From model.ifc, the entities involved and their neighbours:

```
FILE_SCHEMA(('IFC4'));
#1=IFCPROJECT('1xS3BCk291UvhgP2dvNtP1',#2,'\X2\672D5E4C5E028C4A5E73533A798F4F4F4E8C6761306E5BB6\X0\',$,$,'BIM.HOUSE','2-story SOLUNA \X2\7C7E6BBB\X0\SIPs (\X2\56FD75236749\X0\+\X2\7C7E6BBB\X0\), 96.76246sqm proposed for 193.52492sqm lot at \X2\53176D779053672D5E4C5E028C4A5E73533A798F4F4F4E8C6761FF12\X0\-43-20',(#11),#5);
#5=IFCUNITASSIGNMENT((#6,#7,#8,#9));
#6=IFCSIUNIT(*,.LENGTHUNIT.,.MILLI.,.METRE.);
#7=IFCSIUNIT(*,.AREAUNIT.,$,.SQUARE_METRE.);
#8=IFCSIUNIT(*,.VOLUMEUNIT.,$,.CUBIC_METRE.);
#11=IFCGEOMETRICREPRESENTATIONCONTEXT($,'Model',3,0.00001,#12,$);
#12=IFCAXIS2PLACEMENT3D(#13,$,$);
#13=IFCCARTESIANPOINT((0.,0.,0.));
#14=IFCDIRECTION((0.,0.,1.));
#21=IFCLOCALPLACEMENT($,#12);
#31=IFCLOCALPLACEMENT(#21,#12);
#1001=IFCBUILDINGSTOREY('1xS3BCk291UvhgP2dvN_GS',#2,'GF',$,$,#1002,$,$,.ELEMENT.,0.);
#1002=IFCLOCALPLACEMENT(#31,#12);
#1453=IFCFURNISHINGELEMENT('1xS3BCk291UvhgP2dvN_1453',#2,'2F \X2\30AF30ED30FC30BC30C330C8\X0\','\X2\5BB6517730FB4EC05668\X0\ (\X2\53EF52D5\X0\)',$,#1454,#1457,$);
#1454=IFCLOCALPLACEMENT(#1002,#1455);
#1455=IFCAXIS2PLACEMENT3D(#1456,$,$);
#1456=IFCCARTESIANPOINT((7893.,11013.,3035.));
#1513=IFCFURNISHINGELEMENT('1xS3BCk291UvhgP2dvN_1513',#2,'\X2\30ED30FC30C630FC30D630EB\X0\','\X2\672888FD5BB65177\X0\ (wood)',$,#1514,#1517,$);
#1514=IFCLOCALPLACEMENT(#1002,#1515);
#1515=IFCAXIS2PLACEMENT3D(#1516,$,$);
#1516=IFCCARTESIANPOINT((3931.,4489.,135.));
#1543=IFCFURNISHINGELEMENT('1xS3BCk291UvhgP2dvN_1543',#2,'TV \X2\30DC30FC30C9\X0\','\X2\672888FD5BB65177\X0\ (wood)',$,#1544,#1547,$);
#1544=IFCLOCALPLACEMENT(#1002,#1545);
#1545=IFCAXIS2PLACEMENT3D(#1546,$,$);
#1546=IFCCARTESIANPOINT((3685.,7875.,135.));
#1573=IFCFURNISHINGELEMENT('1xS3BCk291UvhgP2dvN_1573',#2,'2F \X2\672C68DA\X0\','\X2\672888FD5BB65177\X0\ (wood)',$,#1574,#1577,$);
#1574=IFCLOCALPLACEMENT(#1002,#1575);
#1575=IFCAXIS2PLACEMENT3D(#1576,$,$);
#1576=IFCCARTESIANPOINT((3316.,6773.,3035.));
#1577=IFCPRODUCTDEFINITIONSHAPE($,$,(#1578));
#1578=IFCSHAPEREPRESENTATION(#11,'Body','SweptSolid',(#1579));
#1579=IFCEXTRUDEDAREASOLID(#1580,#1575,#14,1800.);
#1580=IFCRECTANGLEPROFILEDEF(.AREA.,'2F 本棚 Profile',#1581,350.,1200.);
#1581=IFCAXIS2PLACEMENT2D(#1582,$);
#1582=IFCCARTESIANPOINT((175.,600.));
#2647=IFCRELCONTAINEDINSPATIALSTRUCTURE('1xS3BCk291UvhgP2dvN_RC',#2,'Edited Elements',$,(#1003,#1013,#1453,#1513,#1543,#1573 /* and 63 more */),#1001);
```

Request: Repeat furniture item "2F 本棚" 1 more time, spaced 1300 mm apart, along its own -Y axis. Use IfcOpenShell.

```python
import ifcopenshell
import ifcopenshell.api.geometry
import ifcopenshell.api.root
import ifcopenshell.util.element
import ifcopenshell.util.placement
import ifcopenshell.util.unit

model = ifcopenshell.open("model.ifc")
unit_scale = ifcopenshell.util.unit.calculate_unit_scale(model)


def reuse_history(source, copy):
    """copy_class also copies each property set's owner history, people and application; keep the originals."""
    for rel in copy.IsDefinedBy:
        if rel.is_a("IfcRelDefinesByProperties") and (history := rel.RelatingPropertyDefinition.OwnerHistory):
            rel.RelatingPropertyDefinition.OwnerHistory = source.OwnerHistory
            ifcopenshell.util.element.remove_deep2(model, history)


source = model.by_id(1573)
base = ifcopenshell.util.placement.get_local_placement(source.ObjectPlacement)
step = -base[:3, 1] * 1.3 / unit_scale

for i in range(1, 2):
    copy = ifcopenshell.api.root.copy_class(model, product=source)
    copy.Representation = ifcopenshell.util.element.copy_deep(
        model, source.Representation, exclude=["IfcGeometricRepresentationContext", "IfcRepresentationMap"]
    )
    reuse_history(source, copy)
    matrix = base.copy()
    matrix[:3, 3] += i * step
    print("added at", matrix[:3, 3].round(3) + 0.0)
    ifcopenshell.api.geometry.edit_object_placement(model, product=copy, matrix=matrix, is_si=False)

model.write("model_rev.ifc")
```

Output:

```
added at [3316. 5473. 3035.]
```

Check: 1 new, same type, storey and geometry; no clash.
